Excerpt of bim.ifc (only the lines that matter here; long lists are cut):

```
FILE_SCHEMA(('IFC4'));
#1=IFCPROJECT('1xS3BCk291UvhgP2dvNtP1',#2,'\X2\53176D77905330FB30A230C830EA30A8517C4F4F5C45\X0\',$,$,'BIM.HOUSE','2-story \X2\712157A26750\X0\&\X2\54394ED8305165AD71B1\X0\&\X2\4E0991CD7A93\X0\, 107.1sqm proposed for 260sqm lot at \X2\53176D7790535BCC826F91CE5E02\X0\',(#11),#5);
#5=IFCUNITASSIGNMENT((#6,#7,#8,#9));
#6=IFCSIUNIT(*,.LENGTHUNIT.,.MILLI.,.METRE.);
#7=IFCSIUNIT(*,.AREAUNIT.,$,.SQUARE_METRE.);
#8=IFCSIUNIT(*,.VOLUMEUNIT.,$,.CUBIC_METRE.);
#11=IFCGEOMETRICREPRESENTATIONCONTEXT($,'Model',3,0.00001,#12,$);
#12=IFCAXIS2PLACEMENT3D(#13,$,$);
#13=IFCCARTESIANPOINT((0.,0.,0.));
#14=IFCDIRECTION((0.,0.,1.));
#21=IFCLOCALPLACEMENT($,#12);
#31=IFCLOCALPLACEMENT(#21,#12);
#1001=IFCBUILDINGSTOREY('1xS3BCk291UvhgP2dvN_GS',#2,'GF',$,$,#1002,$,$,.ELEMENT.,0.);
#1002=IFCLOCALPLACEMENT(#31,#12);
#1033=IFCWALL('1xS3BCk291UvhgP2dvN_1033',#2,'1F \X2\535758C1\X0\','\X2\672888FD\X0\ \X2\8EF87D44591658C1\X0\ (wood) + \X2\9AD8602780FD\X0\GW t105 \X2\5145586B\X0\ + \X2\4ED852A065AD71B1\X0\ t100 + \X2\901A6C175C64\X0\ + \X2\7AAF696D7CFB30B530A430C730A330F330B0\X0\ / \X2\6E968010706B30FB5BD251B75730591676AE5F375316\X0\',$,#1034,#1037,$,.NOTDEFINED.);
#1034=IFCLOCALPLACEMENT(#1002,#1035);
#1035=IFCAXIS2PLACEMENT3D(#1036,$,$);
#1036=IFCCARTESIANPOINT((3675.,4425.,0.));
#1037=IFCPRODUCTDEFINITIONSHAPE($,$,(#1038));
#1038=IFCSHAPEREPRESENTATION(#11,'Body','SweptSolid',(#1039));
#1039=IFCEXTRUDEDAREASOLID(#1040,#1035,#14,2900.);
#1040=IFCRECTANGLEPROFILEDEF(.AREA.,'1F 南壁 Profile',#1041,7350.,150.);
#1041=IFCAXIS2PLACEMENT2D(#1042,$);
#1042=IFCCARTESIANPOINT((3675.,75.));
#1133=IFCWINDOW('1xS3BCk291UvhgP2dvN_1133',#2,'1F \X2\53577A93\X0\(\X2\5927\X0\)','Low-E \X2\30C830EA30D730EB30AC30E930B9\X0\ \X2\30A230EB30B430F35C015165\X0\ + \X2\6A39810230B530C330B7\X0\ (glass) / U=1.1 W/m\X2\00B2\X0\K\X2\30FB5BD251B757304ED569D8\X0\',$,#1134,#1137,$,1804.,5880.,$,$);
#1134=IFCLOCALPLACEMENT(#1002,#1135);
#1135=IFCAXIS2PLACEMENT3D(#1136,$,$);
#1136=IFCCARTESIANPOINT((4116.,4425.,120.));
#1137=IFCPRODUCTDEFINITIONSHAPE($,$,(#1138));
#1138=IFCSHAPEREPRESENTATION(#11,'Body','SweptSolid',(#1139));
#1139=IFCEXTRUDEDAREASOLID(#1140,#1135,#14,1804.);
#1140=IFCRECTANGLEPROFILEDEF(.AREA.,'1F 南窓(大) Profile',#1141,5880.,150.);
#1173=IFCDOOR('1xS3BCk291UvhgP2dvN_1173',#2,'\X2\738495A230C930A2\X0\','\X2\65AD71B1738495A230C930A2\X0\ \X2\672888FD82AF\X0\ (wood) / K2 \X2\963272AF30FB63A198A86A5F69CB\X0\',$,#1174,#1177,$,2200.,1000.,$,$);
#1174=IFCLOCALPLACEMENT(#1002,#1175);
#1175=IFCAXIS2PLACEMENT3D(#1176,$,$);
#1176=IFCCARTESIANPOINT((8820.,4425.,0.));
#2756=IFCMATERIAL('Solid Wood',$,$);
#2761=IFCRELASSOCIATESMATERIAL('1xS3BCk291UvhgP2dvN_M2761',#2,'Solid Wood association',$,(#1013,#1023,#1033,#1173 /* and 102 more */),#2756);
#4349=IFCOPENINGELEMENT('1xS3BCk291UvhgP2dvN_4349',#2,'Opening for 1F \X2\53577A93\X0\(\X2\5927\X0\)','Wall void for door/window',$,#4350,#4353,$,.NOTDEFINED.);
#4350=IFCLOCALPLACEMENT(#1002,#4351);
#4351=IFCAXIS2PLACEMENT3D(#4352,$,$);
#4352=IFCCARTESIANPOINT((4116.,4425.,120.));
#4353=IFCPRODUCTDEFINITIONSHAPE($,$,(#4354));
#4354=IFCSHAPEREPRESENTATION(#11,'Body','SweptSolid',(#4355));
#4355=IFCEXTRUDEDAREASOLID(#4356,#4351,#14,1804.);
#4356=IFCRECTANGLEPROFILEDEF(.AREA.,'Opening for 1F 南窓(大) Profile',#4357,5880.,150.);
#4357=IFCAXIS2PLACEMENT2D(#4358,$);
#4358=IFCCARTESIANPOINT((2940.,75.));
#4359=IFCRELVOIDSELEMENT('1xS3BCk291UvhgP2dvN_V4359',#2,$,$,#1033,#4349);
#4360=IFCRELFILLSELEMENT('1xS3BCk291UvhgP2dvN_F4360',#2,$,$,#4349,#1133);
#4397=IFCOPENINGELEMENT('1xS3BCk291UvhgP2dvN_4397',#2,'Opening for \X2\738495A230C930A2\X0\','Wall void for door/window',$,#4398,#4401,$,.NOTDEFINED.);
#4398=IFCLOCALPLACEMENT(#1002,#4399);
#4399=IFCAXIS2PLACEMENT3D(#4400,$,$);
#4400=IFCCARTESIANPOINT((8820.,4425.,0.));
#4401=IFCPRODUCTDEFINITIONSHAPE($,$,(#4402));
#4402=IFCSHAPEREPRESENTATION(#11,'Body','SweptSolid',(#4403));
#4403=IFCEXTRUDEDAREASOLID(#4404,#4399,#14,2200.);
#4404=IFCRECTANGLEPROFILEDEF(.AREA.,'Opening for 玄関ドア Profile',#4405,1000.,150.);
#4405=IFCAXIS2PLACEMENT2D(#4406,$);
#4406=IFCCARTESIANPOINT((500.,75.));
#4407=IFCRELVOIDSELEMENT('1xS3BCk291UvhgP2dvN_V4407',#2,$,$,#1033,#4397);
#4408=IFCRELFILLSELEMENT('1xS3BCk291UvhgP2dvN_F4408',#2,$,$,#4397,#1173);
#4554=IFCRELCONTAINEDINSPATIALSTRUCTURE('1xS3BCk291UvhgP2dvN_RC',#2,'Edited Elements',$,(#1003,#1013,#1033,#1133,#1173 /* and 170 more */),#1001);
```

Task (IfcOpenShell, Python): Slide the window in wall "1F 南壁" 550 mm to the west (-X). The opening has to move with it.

```python
import ifcopenshell
import ifcopenshell.api.geometry
import ifcopenshell.util.placement
import ifcopenshell.util.unit

model = ifcopenshell.open("bim.ifc")
unit_scale = ifcopenshell.util.unit.calculate_unit_scale(model)

window = model.by_guid("1xS3BCk291UvhgP2dvN_1133")
opening = window.FillsVoids[0].RelatingOpeningElement
wall = opening.VoidsElements[0].RelatingBuildingElement

wall_matrix = ifcopenshell.util.placement.get_local_placement(wall.ObjectPlacement)
shift = wall_matrix[:3, 0] * -0.55 / unit_scale
before = ifcopenshell.util.placement.get_local_placement(window.ObjectPlacement)[:3, 3].copy()

# The window is not placed relative to its opening, so move both.
for product in (opening, window):
    matrix = ifcopenshell.util.placement.get_local_placement(product.ObjectPlacement)
    matrix[:3, 3] += shift
    ifcopenshell.api.geometry.edit_object_placement(model, product=product, matrix=matrix, is_si=False)

after = ifcopenshell.util.placement.get_local_placement(window.ObjectPlacement)[:3, 3]
print("window moved by", (after - before).round(3) + 0.0)

model.write("bim_updated.ifc")
```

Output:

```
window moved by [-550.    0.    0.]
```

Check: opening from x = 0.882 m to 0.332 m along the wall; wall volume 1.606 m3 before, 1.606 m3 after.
